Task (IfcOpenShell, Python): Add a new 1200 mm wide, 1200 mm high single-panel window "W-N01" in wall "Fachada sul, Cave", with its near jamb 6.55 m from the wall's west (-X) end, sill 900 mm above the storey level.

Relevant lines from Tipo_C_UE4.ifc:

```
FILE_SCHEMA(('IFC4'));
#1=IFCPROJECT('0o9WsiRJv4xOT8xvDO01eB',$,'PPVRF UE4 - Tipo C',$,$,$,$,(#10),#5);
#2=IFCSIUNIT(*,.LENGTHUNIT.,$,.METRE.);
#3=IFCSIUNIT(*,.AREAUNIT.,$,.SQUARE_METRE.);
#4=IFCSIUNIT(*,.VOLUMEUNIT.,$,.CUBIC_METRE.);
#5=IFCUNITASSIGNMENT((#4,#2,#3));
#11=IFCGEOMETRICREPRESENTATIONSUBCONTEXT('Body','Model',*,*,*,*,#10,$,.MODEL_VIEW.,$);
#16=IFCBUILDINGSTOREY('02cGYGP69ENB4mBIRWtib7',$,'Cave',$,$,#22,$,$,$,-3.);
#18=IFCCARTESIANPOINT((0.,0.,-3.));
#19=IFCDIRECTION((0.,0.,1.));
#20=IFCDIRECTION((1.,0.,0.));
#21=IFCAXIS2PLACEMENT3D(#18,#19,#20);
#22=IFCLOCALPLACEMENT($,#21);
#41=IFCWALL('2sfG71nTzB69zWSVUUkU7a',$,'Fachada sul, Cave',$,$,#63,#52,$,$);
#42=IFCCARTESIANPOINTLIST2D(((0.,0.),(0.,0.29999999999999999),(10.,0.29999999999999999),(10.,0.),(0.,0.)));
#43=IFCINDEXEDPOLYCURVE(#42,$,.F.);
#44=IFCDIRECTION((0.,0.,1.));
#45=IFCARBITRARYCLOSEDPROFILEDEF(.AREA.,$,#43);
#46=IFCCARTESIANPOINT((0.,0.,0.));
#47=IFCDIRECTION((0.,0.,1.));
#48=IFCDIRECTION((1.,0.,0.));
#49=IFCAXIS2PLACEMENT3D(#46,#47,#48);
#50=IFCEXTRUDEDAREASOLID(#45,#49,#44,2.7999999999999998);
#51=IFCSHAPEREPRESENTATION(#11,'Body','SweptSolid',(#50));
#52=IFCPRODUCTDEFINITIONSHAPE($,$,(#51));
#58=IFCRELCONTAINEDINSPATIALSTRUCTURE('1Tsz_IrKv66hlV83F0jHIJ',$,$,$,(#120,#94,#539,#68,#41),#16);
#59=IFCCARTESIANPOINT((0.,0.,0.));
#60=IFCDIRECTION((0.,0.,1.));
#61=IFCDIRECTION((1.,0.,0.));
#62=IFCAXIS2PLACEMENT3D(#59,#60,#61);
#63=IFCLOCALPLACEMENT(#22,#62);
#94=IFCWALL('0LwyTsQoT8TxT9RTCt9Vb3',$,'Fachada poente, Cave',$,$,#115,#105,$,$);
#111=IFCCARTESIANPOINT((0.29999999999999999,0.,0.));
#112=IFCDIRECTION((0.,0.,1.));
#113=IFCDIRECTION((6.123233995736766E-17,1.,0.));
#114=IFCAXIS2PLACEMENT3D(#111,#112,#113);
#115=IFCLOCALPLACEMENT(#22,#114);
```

```python
import numpy as np
import ifcopenshell
import ifcopenshell.api.feature
import ifcopenshell.api.geometry
import ifcopenshell.api.root
import ifcopenshell.api.spatial
import ifcopenshell.geom
import ifcopenshell.util.element
import ifcopenshell.util.placement
import ifcopenshell.util.representation
import ifcopenshell.util.shape
import ifcopenshell.util.unit

model = ifcopenshell.open("Tipo_C_UE4.ifc")
unit_scale = ifcopenshell.util.unit.calculate_unit_scale(model)
settings = ifcopenshell.geom.settings()


def volume(element):
    """Net volume in cubic metres, openings subtracted."""
    shape = ifcopenshell.geom.create_shape(settings, element)
    return ifcopenshell.util.shape.get_volume(shape.geometry)


wall = model.by_id(41)
storey = ifcopenshell.util.element.get_container(wall, ifc_class="IfcBuildingStorey")
context = ifcopenshell.util.representation.get_context(model, "Model", "Body", "MODEL_VIEW")
before = volume(wall)

width, height, from_end, sill = 1.2, 1.2, 6.55, 0.9  # metres

# The wall runs along its own X axis, and the end named is its -X end.
wall_shape = ifcopenshell.geom.create_shape(settings, wall)
x, y, z = ifcopenshell.util.shape.get_vertices(wall_shape.geometry).T
start = x.min() + from_end
face, thickness = float(y.min()), float(y.max() - y.min())
wall_matrix = ifcopenshell.util.placement.get_local_placement(wall.ObjectPlacement)
level = ifcopenshell.util.placement.get_local_placement(storey.ObjectPlacement)[2, 3]


def in_wall(x, y):
    """Placement at x, y metres in the wall's axes, at sill height."""
    matrix = wall_matrix.copy()
    matrix[:, 3] = wall_matrix @ np.array([x / unit_scale, y / unit_scale, 0.0, 1.0])
    matrix[2, 3] = level + sill / unit_scale
    return matrix


# Opening: a box that overshoots both wall faces by 50 mm.
opening = ifcopenshell.api.root.create_entity(model, ifc_class="IfcOpeningElement", predefined_type="OPENING")
box = ifcopenshell.api.geometry.add_wall_representation(
    model, context=context, length=width, height=height, thickness=thickness + 0.1
)
ifcopenshell.api.geometry.assign_representation(model, product=opening, representation=box)
ifcopenshell.api.geometry.edit_object_placement(model, product=opening, matrix=in_wall(start, face - 0.05), is_si=False)
ifcopenshell.api.feature.add_feature(model, feature=opening, element=wall)

window = ifcopenshell.api.root.create_entity(model, ifc_class="IfcWindow", name="W-N01", predefined_type="WINDOW")
window.OverallWidth, window.OverallHeight = width / unit_scale, height / unit_scale
window.PartitioningType = "SINGLE_PANEL"
body = ifcopenshell.api.geometry.add_window_representation(
    model,
    context=context,
    overall_width=window.OverallWidth,
    overall_height=window.OverallHeight,
    partition_type="SINGLE_PANEL",
)
ifcopenshell.api.geometry.assign_representation(model, product=window, representation=body)
ifcopenshell.api.spatial.assign_container(model, products=[window], relating_structure=storey)
ifcopenshell.api.feature.add_filling(model, opening=opening, element=window)

# Centre the window in the wall's thickness.
ifcopenshell.api.geometry.edit_object_placement(model, product=window, matrix=in_wall(start, face), is_si=False)
window_shape = ifcopenshell.geom.create_shape(settings, window)
depth = ifcopenshell.util.shape.get_vertices(window_shape.geometry)[:, 1]
offset = face + thickness / 2 - (depth.min() + depth.max()) / 2
ifcopenshell.api.geometry.edit_object_placement(model, product=window, matrix=in_wall(start, offset), is_si=False)

after = volume(wall)

print(f"wall volume {before:.3f} -> {after:.3f} m3")

model.write("Tipo_C_UE4_edited.ifc")
```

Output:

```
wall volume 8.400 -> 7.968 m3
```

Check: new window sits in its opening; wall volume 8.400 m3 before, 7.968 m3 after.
